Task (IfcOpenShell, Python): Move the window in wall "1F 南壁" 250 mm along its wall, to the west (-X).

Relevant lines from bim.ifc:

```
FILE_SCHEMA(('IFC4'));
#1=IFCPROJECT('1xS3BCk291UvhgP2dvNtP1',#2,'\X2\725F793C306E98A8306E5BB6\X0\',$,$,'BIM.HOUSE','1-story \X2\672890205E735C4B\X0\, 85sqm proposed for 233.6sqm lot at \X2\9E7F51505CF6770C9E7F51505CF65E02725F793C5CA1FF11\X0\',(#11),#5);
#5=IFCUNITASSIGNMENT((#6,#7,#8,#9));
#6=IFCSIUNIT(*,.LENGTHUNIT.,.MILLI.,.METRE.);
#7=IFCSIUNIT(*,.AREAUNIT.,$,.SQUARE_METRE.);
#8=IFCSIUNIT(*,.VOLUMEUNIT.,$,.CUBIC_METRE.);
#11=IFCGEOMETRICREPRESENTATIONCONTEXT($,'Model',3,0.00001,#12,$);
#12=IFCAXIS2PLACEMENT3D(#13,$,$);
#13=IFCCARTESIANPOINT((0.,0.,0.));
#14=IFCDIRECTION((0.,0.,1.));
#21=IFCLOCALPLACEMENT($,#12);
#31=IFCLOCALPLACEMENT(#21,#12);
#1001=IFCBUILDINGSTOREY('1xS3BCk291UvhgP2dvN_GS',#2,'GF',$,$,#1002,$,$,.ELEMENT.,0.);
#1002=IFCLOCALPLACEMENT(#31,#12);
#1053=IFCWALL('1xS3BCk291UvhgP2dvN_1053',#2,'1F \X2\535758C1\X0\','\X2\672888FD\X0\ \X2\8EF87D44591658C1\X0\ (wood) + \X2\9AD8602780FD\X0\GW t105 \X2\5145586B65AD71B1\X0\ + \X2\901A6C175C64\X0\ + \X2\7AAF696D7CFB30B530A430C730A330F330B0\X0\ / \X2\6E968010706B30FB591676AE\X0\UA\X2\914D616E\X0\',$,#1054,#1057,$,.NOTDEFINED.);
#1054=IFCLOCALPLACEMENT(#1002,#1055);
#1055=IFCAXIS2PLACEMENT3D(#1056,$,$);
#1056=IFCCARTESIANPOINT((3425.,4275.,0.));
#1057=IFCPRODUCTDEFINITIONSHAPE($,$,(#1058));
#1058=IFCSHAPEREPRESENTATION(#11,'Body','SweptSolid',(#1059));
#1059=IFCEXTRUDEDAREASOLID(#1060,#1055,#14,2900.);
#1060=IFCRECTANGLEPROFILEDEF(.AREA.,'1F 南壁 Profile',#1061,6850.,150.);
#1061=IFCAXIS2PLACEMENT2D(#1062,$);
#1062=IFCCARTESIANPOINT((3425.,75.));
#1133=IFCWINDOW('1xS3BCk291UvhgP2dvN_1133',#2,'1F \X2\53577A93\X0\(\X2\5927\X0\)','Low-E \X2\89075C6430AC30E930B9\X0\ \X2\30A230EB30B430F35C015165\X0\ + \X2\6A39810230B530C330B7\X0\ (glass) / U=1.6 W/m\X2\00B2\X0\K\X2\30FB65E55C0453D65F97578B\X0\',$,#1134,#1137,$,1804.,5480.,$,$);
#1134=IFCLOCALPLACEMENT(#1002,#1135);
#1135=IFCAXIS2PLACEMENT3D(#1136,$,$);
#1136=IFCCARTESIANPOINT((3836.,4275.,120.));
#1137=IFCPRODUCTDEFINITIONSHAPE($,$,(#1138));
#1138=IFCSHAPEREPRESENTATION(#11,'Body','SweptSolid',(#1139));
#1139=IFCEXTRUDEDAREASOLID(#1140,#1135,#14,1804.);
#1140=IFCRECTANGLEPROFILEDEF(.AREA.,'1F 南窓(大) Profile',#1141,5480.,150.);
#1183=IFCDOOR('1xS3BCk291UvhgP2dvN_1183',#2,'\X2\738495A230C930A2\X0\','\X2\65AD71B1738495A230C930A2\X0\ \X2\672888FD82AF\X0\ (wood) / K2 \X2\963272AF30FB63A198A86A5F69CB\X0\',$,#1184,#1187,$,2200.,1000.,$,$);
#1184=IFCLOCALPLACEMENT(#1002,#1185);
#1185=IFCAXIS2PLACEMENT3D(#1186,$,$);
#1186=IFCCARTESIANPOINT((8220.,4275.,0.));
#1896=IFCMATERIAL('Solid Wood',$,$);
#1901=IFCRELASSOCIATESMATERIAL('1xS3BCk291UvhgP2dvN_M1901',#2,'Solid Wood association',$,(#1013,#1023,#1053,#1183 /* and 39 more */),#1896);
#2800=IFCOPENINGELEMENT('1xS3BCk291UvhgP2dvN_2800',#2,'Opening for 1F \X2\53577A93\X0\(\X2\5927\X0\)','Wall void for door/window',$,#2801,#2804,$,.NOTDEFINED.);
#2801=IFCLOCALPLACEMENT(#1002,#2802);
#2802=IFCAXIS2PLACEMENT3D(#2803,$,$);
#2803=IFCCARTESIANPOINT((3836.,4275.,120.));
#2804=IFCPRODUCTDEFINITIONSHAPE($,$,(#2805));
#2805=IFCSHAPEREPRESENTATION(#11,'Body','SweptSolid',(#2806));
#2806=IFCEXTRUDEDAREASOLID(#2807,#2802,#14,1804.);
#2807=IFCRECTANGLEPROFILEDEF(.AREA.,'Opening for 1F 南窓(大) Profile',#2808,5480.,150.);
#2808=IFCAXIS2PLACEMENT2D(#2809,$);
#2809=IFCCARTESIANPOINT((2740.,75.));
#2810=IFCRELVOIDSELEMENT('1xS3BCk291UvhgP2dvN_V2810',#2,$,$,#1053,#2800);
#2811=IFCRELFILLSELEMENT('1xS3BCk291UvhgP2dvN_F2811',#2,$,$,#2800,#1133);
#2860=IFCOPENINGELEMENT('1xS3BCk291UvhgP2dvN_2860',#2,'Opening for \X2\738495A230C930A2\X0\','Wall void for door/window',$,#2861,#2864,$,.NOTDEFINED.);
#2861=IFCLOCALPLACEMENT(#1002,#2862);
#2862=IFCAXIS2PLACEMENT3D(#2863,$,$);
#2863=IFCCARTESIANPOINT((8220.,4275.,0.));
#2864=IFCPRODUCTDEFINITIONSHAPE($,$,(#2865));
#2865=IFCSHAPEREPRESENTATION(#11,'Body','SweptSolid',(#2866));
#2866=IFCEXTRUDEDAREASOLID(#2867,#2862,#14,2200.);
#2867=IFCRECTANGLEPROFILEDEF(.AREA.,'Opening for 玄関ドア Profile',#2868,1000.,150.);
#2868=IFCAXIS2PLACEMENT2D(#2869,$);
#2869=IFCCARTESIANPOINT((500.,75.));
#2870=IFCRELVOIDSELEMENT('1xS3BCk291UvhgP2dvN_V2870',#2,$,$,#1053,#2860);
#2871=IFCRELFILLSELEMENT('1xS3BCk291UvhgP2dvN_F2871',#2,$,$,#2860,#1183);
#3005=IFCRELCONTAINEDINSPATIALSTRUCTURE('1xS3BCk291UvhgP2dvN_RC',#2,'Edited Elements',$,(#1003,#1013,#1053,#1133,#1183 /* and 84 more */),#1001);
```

```python
import ifcopenshell
import ifcopenshell.api.geometry
import ifcopenshell.util.placement
import ifcopenshell.util.unit

model = ifcopenshell.open("bim.ifc")
unit_scale = ifcopenshell.util.unit.calculate_unit_scale(model)

window = model.by_guid("1xS3BCk291UvhgP2dvN_1133")
opening = window.FillsVoids[0].RelatingOpeningElement
wall = opening.VoidsElements[0].RelatingBuildingElement

wall_matrix = ifcopenshell.util.placement.get_local_placement(wall.ObjectPlacement)
shift = wall_matrix[:3, 0] * -0.25 / unit_scale
before = ifcopenshell.util.placement.get_local_placement(window.ObjectPlacement)[:3, 3].copy()

# The window is not placed relative to its opening, so move both.
for product in (opening, window):
    matrix = ifcopenshell.util.placement.get_local_placement(product.ObjectPlacement)
    matrix[:3, 3] += shift
    ifcopenshell.api.geometry.edit_object_placement(model, product=product, matrix=matrix, is_si=False)

after = ifcopenshell.util.placement.get_local_placement(window.ObjectPlacement)[:3, 3]
print("window moved by", (after - before).round(3) + 0.0)

model.write("bim_updated.ifc")
```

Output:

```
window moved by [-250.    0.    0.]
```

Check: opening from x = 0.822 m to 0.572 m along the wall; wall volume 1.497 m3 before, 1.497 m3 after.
